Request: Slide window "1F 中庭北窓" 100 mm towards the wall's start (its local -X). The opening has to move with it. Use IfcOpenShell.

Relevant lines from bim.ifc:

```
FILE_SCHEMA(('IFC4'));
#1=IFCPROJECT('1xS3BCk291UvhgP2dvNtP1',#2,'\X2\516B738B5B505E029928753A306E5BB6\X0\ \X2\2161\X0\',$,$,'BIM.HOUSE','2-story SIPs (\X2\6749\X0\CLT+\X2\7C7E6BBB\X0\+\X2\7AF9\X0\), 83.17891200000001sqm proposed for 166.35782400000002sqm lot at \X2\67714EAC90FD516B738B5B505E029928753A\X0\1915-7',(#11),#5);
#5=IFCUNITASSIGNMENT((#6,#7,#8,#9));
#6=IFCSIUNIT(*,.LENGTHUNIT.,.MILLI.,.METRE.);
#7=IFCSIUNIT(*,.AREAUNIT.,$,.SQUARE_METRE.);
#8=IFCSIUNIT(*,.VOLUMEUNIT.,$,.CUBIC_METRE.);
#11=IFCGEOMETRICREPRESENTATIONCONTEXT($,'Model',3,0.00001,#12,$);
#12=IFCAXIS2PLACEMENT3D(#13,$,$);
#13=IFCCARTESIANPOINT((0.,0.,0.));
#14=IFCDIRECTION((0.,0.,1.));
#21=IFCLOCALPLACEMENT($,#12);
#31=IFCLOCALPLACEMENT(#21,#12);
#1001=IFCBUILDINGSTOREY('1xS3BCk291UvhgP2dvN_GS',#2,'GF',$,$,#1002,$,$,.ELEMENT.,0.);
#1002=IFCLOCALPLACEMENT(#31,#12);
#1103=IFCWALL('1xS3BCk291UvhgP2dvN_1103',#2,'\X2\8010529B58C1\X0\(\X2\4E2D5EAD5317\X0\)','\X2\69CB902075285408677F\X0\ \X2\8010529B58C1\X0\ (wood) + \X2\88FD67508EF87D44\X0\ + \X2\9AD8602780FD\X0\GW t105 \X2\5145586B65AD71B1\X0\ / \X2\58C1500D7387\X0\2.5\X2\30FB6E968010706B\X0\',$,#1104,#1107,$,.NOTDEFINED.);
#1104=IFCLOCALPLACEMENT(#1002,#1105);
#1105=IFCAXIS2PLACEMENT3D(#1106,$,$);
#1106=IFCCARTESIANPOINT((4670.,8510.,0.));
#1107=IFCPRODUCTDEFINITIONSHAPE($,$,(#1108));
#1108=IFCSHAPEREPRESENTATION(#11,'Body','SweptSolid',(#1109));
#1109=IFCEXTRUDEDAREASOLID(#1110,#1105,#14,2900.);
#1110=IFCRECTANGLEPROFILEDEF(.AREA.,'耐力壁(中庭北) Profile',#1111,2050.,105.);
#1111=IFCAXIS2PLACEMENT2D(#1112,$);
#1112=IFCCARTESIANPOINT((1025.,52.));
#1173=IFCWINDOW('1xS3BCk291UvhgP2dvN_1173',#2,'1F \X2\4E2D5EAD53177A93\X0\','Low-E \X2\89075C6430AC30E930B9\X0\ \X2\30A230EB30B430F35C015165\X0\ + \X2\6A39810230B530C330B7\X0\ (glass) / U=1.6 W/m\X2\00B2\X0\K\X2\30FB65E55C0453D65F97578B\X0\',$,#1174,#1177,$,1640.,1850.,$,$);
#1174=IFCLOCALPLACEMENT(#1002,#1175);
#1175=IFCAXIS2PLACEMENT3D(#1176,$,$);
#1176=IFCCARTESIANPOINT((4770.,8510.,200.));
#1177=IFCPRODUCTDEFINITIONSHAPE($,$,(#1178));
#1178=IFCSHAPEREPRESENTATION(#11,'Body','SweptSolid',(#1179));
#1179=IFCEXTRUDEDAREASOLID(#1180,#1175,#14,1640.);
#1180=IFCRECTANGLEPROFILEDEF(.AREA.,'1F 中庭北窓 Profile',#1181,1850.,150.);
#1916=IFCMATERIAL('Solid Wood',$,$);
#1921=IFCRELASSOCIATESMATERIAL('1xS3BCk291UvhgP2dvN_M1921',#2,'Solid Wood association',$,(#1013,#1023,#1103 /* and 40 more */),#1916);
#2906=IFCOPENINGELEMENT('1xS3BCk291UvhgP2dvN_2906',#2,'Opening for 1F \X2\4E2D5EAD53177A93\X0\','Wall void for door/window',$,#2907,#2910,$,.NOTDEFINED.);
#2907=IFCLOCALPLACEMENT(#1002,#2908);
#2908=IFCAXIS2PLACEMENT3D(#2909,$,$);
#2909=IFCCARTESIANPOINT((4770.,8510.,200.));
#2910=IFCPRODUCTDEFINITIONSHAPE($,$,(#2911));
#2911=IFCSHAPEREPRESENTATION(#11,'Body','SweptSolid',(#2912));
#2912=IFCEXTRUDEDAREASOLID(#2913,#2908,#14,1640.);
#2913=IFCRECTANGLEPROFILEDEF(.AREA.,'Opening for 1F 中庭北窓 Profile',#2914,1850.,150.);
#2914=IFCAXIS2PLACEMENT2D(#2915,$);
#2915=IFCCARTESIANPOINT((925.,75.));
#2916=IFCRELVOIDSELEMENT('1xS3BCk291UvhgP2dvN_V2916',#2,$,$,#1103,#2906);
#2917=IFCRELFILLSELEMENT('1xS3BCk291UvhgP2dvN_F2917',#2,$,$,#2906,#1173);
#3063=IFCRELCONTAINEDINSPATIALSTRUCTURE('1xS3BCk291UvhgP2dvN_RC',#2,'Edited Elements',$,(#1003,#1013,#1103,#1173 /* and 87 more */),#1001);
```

```python
import ifcopenshell
import ifcopenshell.api.geometry
import ifcopenshell.util.placement

model = ifcopenshell.open("bim.ifc")

window = model.by_guid("1xS3BCk291UvhgP2dvN_1173")
opening = window.FillsVoids[0].RelatingOpeningElement
wall = opening.VoidsElements[0].RelatingBuildingElement

wall_matrix = ifcopenshell.util.placement.get_local_placement(wall.ObjectPlacement)
shift = wall_matrix[:3, 0] * -100.0
before = ifcopenshell.util.placement.get_local_placement(window.ObjectPlacement)[:3, 3].copy()

# The window is not placed relative to its opening, so move both.
for product in (opening, window):
    matrix = ifcopenshell.util.placement.get_local_placement(product.ObjectPlacement)
    matrix[:3, 3] += shift
    ifcopenshell.api.geometry.edit_object_placement(model, product=product, matrix=matrix, is_si=False)

after = ifcopenshell.util.placement.get_local_placement(window.ObjectPlacement)[:3, 3]
print("window moved by", (after - before).round(3) + 0.0)

model.write("bim_v2.ifc")
```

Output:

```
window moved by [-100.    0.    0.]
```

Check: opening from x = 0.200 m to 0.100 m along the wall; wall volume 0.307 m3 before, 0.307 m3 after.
